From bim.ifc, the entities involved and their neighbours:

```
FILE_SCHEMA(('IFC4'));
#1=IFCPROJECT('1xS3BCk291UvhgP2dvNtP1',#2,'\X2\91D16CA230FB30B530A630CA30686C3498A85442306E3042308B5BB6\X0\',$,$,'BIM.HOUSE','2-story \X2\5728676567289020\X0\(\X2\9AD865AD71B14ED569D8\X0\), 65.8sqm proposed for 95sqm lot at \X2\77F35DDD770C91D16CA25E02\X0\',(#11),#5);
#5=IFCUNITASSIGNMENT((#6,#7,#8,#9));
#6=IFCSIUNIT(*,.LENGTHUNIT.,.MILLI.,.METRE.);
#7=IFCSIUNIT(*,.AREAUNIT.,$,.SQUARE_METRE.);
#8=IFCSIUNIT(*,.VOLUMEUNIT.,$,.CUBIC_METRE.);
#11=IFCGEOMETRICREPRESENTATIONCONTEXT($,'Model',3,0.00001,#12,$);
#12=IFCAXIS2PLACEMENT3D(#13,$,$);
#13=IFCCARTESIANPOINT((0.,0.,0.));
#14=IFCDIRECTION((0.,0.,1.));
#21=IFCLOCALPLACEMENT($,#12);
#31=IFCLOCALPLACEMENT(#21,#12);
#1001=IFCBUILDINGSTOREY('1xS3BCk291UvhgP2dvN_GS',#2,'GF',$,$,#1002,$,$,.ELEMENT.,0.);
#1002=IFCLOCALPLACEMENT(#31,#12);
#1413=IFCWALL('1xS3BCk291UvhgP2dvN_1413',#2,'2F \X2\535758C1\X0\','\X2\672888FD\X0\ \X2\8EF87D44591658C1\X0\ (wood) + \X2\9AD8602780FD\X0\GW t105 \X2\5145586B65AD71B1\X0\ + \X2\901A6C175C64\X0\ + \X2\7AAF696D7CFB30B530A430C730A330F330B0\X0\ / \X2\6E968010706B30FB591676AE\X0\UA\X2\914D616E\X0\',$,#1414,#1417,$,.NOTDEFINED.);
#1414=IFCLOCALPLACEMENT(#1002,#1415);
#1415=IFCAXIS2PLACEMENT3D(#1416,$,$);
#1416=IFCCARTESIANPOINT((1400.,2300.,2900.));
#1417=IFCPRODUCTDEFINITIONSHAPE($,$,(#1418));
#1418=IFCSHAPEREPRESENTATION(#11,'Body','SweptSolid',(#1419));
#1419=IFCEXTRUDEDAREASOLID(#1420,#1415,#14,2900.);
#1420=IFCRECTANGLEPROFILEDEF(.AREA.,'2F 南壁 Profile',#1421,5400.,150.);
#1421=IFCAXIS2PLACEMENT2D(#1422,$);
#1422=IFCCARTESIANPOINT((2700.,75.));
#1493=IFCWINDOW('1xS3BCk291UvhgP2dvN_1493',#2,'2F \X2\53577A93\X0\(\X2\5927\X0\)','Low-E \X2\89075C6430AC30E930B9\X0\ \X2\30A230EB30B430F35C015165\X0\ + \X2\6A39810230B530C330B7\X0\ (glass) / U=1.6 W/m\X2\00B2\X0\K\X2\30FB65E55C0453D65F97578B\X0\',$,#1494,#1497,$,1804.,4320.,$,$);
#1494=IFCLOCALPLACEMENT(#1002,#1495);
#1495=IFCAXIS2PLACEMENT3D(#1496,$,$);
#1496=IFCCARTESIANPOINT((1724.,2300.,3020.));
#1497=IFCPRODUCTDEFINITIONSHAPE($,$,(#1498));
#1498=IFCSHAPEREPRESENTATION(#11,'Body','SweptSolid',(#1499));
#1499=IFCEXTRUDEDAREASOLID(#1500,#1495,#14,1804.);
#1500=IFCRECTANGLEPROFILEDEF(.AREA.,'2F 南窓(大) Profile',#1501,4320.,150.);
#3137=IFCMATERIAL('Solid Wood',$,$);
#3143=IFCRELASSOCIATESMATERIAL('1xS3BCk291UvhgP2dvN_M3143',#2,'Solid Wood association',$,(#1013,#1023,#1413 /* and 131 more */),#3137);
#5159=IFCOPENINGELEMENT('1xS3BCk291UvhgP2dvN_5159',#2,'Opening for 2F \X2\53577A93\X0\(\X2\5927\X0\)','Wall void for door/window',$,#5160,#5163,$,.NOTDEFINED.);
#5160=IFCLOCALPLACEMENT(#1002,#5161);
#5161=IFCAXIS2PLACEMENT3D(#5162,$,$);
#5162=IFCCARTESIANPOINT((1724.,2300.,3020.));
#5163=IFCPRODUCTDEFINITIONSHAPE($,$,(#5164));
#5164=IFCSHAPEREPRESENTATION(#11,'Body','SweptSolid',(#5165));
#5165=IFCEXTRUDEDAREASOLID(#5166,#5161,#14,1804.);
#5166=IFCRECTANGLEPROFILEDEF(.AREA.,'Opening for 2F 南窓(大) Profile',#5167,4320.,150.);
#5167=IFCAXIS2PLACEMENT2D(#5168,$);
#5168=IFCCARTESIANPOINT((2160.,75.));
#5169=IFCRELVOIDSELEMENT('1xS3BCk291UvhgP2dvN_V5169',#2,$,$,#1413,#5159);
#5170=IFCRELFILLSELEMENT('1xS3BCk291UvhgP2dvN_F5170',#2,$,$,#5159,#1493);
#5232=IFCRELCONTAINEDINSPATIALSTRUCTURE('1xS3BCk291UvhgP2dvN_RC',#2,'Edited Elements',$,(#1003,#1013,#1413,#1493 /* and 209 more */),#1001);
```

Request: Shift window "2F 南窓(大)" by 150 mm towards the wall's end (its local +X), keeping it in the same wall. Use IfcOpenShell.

```python
import ifcopenshell
import ifcopenshell.api.geometry
import ifcopenshell.util.placement
import ifcopenshell.util.unit

model = ifcopenshell.open("bim.ifc")
unit_scale = ifcopenshell.util.unit.calculate_unit_scale(model)

window = model.by_guid("1xS3BCk291UvhgP2dvN_1493")
opening = window.FillsVoids[0].RelatingOpeningElement
wall = opening.VoidsElements[0].RelatingBuildingElement

wall_matrix = ifcopenshell.util.placement.get_local_placement(wall.ObjectPlacement)
shift = wall_matrix[:3, 0] * 0.15 / unit_scale
before = ifcopenshell.util.placement.get_local_placement(window.ObjectPlacement)[:3, 3].copy()

# The window is not placed relative to its opening, so move both.
for product in (opening, window):
    matrix = ifcopenshell.util.placement.get_local_placement(product.ObjectPlacement)
    matrix[:3, 3] += shift
    ifcopenshell.api.geometry.edit_object_placement(model, product=product, matrix=matrix, is_si=False)

after = ifcopenshell.util.placement.get_local_placement(window.ObjectPlacement)[:3, 3]
print("window moved by", (after - before).round(3) + 0.0)

model.write("bim_v2.ifc")
```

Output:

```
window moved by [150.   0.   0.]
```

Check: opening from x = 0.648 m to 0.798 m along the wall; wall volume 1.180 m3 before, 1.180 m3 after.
